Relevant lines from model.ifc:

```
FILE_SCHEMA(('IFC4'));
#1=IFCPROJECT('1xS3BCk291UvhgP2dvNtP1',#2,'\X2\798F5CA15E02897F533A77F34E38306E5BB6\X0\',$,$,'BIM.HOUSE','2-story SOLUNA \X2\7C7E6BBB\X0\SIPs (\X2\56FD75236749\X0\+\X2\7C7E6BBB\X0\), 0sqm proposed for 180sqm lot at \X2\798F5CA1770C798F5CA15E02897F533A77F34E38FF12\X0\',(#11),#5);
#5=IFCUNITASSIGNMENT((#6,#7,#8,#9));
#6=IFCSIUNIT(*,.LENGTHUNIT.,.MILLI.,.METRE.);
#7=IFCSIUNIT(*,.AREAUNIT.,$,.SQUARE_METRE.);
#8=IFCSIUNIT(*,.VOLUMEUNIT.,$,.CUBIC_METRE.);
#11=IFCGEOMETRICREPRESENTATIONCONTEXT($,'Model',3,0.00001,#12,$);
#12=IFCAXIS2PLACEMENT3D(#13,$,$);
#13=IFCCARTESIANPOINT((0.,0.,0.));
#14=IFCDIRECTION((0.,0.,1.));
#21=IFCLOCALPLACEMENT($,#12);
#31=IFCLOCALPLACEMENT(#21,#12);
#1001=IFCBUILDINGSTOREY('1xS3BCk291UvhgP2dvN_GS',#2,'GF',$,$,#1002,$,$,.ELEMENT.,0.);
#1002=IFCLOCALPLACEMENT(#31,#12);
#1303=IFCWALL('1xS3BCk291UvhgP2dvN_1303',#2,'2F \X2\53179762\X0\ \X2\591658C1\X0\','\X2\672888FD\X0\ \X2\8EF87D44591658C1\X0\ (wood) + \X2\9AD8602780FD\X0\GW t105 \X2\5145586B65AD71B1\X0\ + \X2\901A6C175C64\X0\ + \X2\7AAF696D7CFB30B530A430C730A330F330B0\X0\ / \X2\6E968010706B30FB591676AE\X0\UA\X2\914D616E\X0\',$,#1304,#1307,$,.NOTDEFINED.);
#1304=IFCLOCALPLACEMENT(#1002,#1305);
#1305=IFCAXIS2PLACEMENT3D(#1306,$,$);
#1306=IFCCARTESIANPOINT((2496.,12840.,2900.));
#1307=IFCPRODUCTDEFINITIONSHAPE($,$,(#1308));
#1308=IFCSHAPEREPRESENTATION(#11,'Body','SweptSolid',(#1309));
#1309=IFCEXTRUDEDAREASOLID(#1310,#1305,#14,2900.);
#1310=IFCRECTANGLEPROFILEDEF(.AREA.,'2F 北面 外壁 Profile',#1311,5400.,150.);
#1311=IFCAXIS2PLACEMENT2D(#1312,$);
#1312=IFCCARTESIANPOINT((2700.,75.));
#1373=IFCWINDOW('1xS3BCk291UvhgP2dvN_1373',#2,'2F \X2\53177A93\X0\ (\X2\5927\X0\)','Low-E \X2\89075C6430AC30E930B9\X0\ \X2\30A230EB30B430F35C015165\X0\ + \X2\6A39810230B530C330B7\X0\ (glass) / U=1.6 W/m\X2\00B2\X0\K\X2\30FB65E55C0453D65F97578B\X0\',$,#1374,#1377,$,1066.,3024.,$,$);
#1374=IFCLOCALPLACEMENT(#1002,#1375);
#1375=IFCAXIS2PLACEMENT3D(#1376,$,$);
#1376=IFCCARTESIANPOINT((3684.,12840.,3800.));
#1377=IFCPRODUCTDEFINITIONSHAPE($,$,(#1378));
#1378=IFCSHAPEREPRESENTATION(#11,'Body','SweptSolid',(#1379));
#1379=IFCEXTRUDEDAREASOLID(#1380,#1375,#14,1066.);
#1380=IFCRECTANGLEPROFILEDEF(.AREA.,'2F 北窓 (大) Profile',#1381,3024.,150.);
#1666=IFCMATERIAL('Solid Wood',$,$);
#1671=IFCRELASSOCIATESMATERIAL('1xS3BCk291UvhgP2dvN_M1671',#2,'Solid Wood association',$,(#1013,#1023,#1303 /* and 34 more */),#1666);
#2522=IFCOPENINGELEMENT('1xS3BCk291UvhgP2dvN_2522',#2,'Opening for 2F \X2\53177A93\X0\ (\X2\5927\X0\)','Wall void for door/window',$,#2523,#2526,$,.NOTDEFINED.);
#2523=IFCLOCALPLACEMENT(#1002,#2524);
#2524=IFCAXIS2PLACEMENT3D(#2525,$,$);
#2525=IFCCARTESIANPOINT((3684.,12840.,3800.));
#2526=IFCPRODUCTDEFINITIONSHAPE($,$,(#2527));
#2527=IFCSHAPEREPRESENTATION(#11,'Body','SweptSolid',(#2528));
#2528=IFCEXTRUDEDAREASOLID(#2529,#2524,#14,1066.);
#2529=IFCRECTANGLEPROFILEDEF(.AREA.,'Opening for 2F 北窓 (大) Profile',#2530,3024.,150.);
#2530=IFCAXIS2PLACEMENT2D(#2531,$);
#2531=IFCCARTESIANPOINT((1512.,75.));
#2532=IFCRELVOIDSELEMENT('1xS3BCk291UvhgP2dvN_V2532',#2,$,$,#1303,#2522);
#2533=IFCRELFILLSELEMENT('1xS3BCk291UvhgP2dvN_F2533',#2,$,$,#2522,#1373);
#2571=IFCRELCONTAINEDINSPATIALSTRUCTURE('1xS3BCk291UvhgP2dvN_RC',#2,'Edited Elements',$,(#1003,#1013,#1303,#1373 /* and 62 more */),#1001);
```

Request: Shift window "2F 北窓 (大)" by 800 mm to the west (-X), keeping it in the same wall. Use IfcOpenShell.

```python
import ifcopenshell
import ifcopenshell.api.geometry
import ifcopenshell.util.placement

model = ifcopenshell.open("model.ifc")

window = model.by_guid("1xS3BCk291UvhgP2dvN_1373")
opening = window.FillsVoids[0].RelatingOpeningElement
wall = opening.VoidsElements[0].RelatingBuildingElement

wall_matrix = ifcopenshell.util.placement.get_local_placement(wall.ObjectPlacement)
shift = wall_matrix[:3, 0] * -800.0
before = ifcopenshell.util.placement.get_local_placement(window.ObjectPlacement)[:3, 3].copy()

# The window is not placed relative to its opening, so move both.
for product in (opening, window):
    matrix = ifcopenshell.util.placement.get_local_placement(product.ObjectPlacement)
    matrix[:3, 3] += shift
    ifcopenshell.api.geometry.edit_object_placement(model, product=product, matrix=matrix, is_si=False)

after = ifcopenshell.util.placement.get_local_placement(window.ObjectPlacement)[:3, 3]
print("window moved by", (after - before).round(3) + 0.0)

model.write("model_edited.ifc")
```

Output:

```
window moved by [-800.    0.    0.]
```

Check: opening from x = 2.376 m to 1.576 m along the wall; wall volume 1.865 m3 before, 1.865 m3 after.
